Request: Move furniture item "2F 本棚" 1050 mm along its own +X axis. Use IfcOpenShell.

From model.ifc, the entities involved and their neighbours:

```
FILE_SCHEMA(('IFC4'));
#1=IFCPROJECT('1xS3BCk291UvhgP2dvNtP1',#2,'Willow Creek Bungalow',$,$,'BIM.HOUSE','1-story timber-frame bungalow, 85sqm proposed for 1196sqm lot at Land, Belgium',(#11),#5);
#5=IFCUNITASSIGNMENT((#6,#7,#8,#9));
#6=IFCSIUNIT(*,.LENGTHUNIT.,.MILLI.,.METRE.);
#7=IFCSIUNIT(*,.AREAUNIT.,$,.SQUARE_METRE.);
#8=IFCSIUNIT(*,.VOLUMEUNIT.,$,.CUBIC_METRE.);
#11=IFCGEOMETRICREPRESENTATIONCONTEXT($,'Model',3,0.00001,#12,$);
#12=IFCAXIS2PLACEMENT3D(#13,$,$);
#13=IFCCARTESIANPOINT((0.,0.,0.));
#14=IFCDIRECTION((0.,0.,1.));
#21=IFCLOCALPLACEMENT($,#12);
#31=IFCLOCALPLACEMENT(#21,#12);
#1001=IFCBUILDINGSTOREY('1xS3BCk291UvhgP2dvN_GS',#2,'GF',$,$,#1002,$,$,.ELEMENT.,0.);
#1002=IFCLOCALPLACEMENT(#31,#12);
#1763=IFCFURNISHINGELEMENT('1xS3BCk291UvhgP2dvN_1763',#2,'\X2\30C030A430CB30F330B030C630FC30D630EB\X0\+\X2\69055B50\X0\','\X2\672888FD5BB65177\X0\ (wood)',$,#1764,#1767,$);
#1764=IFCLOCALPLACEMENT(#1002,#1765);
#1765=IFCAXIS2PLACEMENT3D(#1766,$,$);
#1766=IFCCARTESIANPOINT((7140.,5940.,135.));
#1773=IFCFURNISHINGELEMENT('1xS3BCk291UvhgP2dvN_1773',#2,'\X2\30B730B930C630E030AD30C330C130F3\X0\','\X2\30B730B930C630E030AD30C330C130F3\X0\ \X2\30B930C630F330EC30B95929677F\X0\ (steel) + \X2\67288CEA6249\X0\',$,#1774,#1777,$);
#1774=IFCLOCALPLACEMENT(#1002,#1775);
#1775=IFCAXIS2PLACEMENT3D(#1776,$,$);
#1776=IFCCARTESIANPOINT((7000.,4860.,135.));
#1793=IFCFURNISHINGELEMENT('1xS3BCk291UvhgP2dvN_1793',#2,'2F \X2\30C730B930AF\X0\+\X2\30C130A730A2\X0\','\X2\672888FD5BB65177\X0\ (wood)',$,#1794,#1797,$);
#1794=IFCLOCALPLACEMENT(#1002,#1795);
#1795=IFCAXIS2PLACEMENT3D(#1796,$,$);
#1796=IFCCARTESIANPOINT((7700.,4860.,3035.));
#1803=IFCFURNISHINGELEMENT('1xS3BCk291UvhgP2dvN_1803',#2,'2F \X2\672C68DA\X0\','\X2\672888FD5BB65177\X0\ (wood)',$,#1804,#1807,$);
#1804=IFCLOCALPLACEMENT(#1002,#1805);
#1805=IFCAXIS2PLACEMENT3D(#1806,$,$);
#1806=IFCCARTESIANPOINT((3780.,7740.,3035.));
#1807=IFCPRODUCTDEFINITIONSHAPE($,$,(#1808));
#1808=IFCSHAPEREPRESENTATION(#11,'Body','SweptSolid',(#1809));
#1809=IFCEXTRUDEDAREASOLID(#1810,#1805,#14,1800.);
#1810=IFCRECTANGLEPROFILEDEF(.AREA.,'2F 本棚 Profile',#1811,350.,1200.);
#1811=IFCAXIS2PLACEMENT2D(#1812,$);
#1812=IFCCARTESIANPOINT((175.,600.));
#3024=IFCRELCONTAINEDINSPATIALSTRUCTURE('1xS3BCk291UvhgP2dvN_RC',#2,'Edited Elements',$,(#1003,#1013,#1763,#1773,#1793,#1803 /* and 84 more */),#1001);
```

```python
import ifcopenshell
import ifcopenshell.api.geometry
import ifcopenshell.util.placement
import ifcopenshell.util.unit

model = ifcopenshell.open("model.ifc")
unit_scale = ifcopenshell.util.unit.calculate_unit_scale(model)

item = model.by_guid("1xS3BCk291UvhgP2dvN_1803")
matrix = ifcopenshell.util.placement.get_local_placement(item.ObjectPlacement)
matrix[:3, 3] += matrix[:3, 0] * 1.05 / unit_scale
ifcopenshell.api.geometry.edit_object_placement(model, product=item, matrix=matrix, is_si=False)

print(ifcopenshell.util.placement.get_local_placement(item.ObjectPlacement).round(3) + 0.0)

model.write("model_rev.ifc")
```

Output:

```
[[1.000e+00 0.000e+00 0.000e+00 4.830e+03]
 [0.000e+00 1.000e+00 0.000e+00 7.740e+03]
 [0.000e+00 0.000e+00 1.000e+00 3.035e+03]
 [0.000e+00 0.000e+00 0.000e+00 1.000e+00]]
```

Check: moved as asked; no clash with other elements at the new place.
